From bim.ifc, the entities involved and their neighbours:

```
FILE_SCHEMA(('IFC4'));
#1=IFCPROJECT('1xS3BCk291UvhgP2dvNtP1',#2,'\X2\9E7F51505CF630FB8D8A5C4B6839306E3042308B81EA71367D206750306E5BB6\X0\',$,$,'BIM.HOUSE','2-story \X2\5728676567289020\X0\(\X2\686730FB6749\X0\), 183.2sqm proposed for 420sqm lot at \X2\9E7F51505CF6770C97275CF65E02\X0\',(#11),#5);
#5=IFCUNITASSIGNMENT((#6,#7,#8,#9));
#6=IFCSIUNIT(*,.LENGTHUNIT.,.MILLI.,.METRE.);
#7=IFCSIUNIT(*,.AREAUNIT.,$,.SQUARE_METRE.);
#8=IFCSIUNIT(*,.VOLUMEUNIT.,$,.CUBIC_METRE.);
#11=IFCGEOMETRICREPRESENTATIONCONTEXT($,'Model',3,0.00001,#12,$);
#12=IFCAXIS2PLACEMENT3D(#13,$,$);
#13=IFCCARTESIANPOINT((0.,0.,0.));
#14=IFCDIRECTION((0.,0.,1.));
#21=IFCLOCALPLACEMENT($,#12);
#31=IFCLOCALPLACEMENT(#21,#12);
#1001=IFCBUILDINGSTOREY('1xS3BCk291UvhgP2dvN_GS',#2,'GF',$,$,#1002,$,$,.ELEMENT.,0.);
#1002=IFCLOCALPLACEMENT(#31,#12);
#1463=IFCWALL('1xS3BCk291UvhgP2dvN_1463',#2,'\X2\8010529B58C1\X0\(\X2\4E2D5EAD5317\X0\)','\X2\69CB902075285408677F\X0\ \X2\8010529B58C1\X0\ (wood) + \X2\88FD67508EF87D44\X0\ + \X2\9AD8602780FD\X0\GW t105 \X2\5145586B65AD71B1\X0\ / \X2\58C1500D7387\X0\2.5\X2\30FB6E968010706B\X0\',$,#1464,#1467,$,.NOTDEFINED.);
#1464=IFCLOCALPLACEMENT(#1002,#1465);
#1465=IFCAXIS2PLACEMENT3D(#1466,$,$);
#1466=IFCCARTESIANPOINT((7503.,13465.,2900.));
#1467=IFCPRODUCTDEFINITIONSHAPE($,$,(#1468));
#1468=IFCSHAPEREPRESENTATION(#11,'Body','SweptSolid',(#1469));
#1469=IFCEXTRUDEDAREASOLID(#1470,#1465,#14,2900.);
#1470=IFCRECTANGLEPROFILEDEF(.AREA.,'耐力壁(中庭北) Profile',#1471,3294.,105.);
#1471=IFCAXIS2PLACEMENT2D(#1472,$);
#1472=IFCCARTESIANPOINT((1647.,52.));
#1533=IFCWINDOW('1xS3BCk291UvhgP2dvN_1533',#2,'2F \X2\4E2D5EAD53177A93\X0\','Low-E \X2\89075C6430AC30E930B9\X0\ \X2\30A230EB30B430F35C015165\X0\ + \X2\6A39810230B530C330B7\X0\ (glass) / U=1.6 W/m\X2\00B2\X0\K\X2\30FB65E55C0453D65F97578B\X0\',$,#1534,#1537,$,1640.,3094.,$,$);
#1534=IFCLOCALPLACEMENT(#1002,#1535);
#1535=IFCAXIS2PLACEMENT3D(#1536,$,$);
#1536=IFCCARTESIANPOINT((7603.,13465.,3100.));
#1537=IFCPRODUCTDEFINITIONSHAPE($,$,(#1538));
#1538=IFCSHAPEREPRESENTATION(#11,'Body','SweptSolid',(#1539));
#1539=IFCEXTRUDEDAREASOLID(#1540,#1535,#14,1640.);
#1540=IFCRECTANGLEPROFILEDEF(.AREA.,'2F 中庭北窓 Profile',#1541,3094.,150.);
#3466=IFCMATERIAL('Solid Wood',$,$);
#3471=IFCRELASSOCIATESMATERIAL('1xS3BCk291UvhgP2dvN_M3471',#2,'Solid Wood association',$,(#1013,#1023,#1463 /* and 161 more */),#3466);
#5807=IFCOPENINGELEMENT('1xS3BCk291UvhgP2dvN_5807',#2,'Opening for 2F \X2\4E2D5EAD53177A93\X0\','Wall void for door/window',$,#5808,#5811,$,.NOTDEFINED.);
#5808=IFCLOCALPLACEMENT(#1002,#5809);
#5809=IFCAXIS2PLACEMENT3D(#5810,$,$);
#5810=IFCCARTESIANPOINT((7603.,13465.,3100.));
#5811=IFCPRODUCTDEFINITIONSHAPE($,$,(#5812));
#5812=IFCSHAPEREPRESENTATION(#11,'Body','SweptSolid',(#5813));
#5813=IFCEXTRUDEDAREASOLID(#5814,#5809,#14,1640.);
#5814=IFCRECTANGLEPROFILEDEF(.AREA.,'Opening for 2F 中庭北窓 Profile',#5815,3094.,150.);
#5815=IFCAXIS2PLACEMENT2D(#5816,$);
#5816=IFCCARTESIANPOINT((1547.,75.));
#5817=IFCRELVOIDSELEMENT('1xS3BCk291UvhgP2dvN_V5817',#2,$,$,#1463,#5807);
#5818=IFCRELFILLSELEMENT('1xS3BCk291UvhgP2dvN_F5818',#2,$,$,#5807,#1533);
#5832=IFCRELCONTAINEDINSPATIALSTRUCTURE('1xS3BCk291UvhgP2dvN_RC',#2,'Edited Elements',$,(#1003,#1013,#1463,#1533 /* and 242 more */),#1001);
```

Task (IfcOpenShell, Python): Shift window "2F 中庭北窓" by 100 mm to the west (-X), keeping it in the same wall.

```python
import ifcopenshell
import ifcopenshell.api.geometry
import ifcopenshell.util.placement

model = ifcopenshell.open("bim.ifc")

window = model.by_id(1533)
opening = window.FillsVoids[0].RelatingOpeningElement
wall = opening.VoidsElements[0].RelatingBuildingElement

wall_matrix = ifcopenshell.util.placement.get_local_placement(wall.ObjectPlacement)
shift = wall_matrix[:3, 0] * -100.0
before = ifcopenshell.util.placement.get_local_placement(window.ObjectPlacement)[:3, 3].copy()

# The window is not placed relative to its opening, so move both.
for product in (opening, window):
    matrix = ifcopenshell.util.placement.get_local_placement(product.ObjectPlacement)
    matrix[:3, 3] += shift
    ifcopenshell.api.geometry.edit_object_placement(model, product=product, matrix=matrix, is_si=False)

after = ifcopenshell.util.placement.get_local_placement(window.ObjectPlacement)[:3, 3]
print("window moved by", (after - before).round(3) + 0.0)

model.write("bim_edited.ifc")
```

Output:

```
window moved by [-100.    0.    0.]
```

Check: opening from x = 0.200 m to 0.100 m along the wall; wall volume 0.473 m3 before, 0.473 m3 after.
